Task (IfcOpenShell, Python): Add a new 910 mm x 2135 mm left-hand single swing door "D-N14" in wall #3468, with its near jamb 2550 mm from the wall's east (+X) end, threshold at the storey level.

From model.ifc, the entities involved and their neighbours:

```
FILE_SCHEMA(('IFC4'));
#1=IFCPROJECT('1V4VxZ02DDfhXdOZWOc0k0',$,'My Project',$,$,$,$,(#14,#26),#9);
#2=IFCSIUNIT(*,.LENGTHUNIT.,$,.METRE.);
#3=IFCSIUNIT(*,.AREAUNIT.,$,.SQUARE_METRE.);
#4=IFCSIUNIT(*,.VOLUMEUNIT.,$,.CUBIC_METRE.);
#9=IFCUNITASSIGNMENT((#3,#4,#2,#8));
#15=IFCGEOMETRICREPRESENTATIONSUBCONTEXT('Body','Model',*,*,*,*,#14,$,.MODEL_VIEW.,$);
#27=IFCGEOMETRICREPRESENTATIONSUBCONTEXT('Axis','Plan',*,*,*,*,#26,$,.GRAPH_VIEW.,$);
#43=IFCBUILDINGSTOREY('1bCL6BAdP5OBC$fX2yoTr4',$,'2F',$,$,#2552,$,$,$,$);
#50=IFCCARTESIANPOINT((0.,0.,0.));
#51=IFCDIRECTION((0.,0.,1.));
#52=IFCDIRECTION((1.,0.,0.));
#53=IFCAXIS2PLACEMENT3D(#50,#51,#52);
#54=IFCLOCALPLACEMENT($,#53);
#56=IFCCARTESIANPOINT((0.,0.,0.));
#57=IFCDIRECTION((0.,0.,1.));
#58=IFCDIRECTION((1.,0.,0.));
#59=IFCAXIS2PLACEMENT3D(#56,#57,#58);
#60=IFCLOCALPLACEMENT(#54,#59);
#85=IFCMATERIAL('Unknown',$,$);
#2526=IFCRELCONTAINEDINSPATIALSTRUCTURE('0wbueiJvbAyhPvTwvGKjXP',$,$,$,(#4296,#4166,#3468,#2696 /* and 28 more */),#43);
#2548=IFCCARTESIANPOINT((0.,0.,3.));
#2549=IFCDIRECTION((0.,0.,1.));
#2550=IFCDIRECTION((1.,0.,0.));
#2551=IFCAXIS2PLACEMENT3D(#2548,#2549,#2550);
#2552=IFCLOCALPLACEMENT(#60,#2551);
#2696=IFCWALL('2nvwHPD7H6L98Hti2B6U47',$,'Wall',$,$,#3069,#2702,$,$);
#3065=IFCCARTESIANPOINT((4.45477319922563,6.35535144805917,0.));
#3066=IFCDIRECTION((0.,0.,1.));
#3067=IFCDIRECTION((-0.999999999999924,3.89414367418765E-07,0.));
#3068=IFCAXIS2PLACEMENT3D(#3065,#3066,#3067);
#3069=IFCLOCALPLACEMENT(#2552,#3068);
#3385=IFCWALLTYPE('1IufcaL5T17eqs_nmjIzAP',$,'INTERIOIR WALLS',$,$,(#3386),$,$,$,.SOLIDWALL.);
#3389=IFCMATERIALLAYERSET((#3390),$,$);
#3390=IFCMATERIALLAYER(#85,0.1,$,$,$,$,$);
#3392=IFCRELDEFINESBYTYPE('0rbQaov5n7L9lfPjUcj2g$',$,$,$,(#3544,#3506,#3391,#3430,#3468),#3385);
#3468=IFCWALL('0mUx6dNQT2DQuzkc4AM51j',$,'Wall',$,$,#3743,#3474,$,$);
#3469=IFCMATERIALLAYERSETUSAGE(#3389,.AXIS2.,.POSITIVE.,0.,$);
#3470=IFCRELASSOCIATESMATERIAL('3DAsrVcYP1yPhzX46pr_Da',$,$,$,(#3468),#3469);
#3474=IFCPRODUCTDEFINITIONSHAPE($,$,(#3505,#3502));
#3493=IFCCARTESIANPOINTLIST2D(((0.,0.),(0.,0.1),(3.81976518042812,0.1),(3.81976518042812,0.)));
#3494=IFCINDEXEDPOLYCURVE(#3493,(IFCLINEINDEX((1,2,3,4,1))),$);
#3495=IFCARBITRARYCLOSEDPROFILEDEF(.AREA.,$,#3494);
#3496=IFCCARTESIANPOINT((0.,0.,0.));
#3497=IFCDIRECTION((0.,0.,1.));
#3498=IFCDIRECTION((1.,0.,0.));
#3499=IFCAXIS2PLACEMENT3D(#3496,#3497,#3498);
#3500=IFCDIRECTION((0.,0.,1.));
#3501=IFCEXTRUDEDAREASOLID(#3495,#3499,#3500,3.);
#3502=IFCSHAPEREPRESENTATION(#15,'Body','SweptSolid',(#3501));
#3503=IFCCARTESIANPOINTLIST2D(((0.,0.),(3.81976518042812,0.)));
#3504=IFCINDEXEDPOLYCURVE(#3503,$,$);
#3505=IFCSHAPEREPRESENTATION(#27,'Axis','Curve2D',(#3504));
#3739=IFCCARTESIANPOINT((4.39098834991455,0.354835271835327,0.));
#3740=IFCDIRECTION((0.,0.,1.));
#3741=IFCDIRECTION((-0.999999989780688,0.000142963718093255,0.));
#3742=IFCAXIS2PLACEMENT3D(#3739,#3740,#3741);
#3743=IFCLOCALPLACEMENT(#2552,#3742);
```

```python
import numpy as np
import ifcopenshell
import ifcopenshell.api.feature
import ifcopenshell.api.geometry
import ifcopenshell.api.root
import ifcopenshell.api.spatial
import ifcopenshell.geom
import ifcopenshell.util.element
import ifcopenshell.util.placement
import ifcopenshell.util.representation
import ifcopenshell.util.shape
import ifcopenshell.util.unit

model = ifcopenshell.open("model.ifc")
unit_scale = ifcopenshell.util.unit.calculate_unit_scale(model)
settings = ifcopenshell.geom.settings()


def volume(element):
    """Net volume in cubic metres, openings subtracted."""
    shape = ifcopenshell.geom.create_shape(settings, element)
    return ifcopenshell.util.shape.get_volume(shape.geometry)


wall = model.by_id(3468)
storey = ifcopenshell.util.element.get_container(wall, ifc_class="IfcBuildingStorey")
context = ifcopenshell.util.representation.get_context(model, "Model", "Body", "MODEL_VIEW")
before = volume(wall)

width, height, from_end, sill = 0.91, 2.135, 2.55, 0.0  # metres

# The wall runs along its own X axis, and the end named is its -X end.
wall_shape = ifcopenshell.geom.create_shape(settings, wall)
x, y, z = ifcopenshell.util.shape.get_vertices(wall_shape.geometry).T
start = x.min() + from_end
face, thickness = float(y.min()), float(y.max() - y.min())
wall_matrix = ifcopenshell.util.placement.get_local_placement(wall.ObjectPlacement)
level = ifcopenshell.util.placement.get_local_placement(storey.ObjectPlacement)[2, 3]


def in_wall(x, y):
    """Placement at x, y metres in the wall's axes, at sill height."""
    matrix = wall_matrix.copy()
    matrix[:, 3] = wall_matrix @ np.array([x / unit_scale, y / unit_scale, 0.0, 1.0])
    matrix[2, 3] = level + sill / unit_scale
    return matrix


# Opening: a box that overshoots both wall faces by 50 mm.
opening = ifcopenshell.api.root.create_entity(model, ifc_class="IfcOpeningElement", predefined_type="OPENING")
box = ifcopenshell.api.geometry.add_wall_representation(
    model, context=context, length=width, height=height, thickness=thickness + 0.1
)
ifcopenshell.api.geometry.assign_representation(model, product=opening, representation=box)
ifcopenshell.api.geometry.edit_object_placement(model, product=opening, matrix=in_wall(start, face - 0.05), is_si=False)
ifcopenshell.api.feature.add_feature(model, feature=opening, element=wall)

door = ifcopenshell.api.root.create_entity(model, ifc_class="IfcDoor", name="D-N14", predefined_type="DOOR")
door.OverallWidth, door.OverallHeight = width / unit_scale, height / unit_scale
door.OperationType = "SINGLE_SWING_LEFT"
body = ifcopenshell.api.geometry.add_door_representation(
    model,
    context=context,
    overall_width=door.OverallWidth,
    overall_height=door.OverallHeight,
    operation_type="SINGLE_SWING_LEFT",
    lining_properties={"LiningDepth": thickness / unit_scale, "ThresholdDepth": thickness / unit_scale},
)
ifcopenshell.api.geometry.assign_representation(model, product=door, representation=body)
ifcopenshell.api.spatial.assign_container(model, products=[door], relating_structure=storey)
ifcopenshell.api.feature.add_filling(model, opening=opening, element=door)

# The lining spans the wall, so the door starts at the wall face.
ifcopenshell.api.geometry.edit_object_placement(model, product=door, matrix=in_wall(start, face), is_si=False)

after = volume(wall)

print(f"wall volume {before:.3f} -> {after:.3f} m3")

model.write("model_v2.ifc")
```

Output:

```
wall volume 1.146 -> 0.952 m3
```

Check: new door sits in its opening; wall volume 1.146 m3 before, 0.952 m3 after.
